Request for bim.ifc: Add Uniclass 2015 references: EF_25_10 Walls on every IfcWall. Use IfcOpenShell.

First a look at what the model holds.

```python
import ifcopenshell

model = ifcopenshell.open("bim.ifc")
print(model.schema)
print("classifications:", [c.Name for c in model.by_type("IfcClassification")])
for ifc_class in ("IfcDoor", "IfcRoof", "IfcStair", "IfcWall", "IfcWindow"):
    print(ifc_class, len(model.by_type(ifc_class)))
```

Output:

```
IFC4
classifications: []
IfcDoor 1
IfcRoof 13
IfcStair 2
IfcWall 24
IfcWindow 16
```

```python
import ifcopenshell
import ifcopenshell.api.classification

model = ifcopenshell.open("bim.ifc")

system = ifcopenshell.api.classification.add_classification(model, classification="Uniclass 2015")

codes = {
    "IfcWall": ("EF_25_10", "Walls"),
}
for ifc_class, (code, name) in codes.items():
    products = model.by_type(ifc_class)
    ifcopenshell.api.classification.add_reference(
        model, products=products, classification=system, identification=code, name=name
    )
    print(code, len(products))

model.write("bim_rev.ifc")
```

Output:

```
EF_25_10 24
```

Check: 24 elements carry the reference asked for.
